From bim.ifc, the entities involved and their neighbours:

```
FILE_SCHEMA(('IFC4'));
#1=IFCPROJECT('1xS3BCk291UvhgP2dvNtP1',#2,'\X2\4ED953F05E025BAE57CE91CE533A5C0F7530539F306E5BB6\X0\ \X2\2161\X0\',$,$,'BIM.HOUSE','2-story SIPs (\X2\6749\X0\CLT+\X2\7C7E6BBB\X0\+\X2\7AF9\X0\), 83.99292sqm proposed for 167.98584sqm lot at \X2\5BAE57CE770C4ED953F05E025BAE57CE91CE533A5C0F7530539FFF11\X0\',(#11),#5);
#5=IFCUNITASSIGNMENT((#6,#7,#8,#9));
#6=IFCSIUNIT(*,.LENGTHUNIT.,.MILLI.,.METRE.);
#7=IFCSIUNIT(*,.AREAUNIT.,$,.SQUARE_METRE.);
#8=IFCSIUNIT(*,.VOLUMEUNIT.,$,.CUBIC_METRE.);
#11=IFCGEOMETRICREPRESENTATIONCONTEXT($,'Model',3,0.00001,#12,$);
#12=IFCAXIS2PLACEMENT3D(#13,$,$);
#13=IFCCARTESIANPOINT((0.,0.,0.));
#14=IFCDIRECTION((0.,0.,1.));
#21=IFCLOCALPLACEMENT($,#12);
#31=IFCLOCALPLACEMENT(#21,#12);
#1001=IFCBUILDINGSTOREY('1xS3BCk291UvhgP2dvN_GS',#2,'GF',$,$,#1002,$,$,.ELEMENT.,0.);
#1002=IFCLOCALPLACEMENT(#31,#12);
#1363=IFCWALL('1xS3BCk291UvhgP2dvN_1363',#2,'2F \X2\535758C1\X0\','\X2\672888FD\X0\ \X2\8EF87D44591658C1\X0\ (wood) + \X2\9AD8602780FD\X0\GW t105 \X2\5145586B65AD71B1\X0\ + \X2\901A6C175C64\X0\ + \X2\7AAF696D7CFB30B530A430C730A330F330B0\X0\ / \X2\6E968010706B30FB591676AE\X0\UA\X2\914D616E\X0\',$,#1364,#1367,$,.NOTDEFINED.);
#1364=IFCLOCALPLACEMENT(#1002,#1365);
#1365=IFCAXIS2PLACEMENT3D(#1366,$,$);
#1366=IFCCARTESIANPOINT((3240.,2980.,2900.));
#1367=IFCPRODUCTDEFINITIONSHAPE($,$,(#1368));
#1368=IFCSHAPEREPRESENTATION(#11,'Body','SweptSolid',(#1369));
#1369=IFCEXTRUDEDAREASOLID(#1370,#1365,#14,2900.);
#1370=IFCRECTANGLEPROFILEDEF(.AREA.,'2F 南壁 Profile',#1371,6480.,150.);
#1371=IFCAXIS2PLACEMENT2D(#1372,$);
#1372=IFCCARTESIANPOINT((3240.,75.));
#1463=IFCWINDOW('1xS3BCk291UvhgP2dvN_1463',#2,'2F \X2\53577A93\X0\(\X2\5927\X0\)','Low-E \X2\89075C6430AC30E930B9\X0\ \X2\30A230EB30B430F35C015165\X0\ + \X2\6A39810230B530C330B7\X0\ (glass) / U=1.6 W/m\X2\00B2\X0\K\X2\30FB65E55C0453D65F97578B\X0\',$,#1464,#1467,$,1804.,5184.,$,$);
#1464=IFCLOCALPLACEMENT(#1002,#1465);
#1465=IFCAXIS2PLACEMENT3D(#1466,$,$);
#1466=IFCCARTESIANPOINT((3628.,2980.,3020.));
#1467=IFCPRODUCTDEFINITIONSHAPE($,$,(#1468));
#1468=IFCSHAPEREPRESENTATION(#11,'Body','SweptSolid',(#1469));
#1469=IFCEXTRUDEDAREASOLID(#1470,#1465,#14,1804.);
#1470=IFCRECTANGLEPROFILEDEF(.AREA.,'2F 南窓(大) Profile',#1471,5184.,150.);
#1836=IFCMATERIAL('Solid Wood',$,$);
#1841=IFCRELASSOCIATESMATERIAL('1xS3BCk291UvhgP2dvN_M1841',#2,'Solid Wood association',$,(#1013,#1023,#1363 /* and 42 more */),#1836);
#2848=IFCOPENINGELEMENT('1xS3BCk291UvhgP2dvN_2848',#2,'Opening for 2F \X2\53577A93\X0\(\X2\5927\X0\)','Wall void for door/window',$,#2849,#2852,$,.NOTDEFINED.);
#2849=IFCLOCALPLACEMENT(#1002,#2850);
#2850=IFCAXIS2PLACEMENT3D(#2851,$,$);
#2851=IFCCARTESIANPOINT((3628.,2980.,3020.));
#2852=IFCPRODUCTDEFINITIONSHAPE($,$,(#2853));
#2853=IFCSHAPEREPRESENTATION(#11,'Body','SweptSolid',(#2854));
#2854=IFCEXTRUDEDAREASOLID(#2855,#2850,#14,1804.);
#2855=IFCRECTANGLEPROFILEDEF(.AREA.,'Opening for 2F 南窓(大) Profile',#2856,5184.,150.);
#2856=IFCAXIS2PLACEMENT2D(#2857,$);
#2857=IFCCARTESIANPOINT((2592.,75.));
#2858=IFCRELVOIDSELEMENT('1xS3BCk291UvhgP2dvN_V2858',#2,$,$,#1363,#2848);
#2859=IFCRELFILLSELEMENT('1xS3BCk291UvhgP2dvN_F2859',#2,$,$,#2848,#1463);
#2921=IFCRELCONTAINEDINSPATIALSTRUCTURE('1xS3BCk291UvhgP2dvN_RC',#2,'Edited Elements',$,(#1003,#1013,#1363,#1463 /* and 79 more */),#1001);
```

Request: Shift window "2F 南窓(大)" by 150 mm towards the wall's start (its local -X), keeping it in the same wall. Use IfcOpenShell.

```python
import ifcopenshell
import ifcopenshell.api.geometry
import ifcopenshell.util.placement
import ifcopenshell.util.unit

model = ifcopenshell.open("bim.ifc")
unit_scale = ifcopenshell.util.unit.calculate_unit_scale(model)

window = model.by_id(1463)
opening = window.FillsVoids[0].RelatingOpeningElement
wall = opening.VoidsElements[0].RelatingBuildingElement

wall_matrix = ifcopenshell.util.placement.get_local_placement(wall.ObjectPlacement)
shift = wall_matrix[:3, 0] * -0.15 / unit_scale
before = ifcopenshell.util.placement.get_local_placement(window.ObjectPlacement)[:3, 3].copy()

# The window is not placed relative to its opening, so move both.
for product in (opening, window):
    matrix = ifcopenshell.util.placement.get_local_placement(product.ObjectPlacement)
    matrix[:3, 3] += shift
    ifcopenshell.api.geometry.edit_object_placement(model, product=product, matrix=matrix, is_si=False)

after = ifcopenshell.util.placement.get_local_placement(window.ObjectPlacement)[:3, 3]
print("window moved by", (after - before).round(3) + 0.0)

model.write("bim-out.ifc")
```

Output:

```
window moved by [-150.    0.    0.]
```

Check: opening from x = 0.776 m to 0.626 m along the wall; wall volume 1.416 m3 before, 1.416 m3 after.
